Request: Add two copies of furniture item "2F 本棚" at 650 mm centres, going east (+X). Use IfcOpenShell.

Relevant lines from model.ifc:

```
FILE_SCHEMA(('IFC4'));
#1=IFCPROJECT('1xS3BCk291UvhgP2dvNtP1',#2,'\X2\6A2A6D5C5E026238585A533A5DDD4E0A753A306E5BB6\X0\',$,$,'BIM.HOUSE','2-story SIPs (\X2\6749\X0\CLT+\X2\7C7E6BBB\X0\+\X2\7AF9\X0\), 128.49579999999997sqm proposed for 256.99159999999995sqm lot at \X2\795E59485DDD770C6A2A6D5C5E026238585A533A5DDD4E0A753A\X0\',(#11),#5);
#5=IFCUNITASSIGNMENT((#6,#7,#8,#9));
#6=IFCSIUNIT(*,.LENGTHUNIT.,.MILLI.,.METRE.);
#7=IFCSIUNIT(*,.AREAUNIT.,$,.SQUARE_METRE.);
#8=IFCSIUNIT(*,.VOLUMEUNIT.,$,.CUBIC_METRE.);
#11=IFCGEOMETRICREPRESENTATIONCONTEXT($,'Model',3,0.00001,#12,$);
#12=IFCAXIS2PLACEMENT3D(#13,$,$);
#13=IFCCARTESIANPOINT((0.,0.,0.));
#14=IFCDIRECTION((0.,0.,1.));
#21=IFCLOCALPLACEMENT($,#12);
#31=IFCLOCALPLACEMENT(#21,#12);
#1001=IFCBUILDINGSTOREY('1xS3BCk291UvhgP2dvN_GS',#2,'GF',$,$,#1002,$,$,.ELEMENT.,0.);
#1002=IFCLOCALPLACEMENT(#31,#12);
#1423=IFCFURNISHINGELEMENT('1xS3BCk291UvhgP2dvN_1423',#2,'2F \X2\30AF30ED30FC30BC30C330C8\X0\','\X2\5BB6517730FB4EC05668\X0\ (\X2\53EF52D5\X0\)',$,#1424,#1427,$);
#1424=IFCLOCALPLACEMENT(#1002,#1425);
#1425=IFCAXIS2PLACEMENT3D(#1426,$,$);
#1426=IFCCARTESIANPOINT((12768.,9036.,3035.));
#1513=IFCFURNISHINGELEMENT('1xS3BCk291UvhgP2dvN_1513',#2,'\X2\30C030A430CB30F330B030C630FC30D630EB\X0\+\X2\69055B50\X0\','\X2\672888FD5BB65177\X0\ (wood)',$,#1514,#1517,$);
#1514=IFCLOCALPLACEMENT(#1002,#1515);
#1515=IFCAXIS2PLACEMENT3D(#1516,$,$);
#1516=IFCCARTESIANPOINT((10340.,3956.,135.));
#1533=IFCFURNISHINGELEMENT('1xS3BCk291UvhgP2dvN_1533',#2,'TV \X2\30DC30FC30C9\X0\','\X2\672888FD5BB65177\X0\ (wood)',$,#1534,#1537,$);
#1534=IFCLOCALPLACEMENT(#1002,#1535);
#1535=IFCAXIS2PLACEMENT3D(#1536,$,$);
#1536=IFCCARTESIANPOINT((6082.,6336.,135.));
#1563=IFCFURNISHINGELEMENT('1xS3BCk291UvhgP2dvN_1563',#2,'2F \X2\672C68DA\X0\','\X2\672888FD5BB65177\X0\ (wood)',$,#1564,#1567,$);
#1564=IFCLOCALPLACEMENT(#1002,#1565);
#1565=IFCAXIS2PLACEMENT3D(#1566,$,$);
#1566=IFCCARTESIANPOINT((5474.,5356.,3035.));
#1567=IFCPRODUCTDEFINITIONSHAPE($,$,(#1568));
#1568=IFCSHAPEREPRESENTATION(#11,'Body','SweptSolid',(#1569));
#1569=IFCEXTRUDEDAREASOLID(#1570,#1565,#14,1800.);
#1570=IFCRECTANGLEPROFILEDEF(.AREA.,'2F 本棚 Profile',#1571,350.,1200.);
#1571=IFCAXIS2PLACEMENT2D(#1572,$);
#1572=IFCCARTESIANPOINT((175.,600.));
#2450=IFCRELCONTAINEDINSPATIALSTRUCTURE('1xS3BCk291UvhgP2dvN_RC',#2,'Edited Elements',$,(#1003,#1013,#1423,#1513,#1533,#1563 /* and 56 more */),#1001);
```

```python
import numpy as np
import ifcopenshell
import ifcopenshell.api.geometry
import ifcopenshell.api.root
import ifcopenshell.util.element
import ifcopenshell.util.placement
import ifcopenshell.util.unit

model = ifcopenshell.open("model.ifc")
unit_scale = ifcopenshell.util.unit.calculate_unit_scale(model)


def reuse_history(source, copy):
    """copy_class also copies each property set's owner history, people and application; keep the originals."""
    for rel in copy.IsDefinedBy:
        if rel.is_a("IfcRelDefinesByProperties") and (history := rel.RelatingPropertyDefinition.OwnerHistory):
            rel.RelatingPropertyDefinition.OwnerHistory = source.OwnerHistory
            ifcopenshell.util.element.remove_deep2(model, history)


source = model.by_guid("1xS3BCk291UvhgP2dvN_1563")
base = ifcopenshell.util.placement.get_local_placement(source.ObjectPlacement)
step = np.array([1.0, 0.0, 0.0]) * 0.65 / unit_scale

for i in range(1, 3):
    copy = ifcopenshell.api.root.copy_class(model, product=source)
    copy.Representation = ifcopenshell.util.element.copy_deep(
        model, source.Representation, exclude=["IfcGeometricRepresentationContext", "IfcRepresentationMap"]
    )
    reuse_history(source, copy)
    matrix = base.copy()
    matrix[:3, 3] += i * step
    print("added at", matrix[:3, 3].round(3) + 0.0)
    ifcopenshell.api.geometry.edit_object_placement(model, product=copy, matrix=matrix, is_si=False)

model.write("model_edited.ifc")
```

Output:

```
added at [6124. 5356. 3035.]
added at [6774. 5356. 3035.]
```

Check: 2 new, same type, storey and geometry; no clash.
